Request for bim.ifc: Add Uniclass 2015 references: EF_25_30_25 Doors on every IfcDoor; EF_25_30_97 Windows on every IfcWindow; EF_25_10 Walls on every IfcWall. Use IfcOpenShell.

First a look at what the model holds.

```python
import ifcopenshell

model = ifcopenshell.open("bim.ifc")
print(model.schema)
print("classifications:", [c.Name for c in model.by_type("IfcClassification")])
for ifc_class in ("IfcDoor", "IfcRoof", "IfcStair", "IfcWall", "IfcWindow"):
    print(ifc_class, len(model.by_type(ifc_class)))
```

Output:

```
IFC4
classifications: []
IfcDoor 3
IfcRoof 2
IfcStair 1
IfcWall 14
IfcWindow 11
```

```python
import ifcopenshell
import ifcopenshell.api.classification

model = ifcopenshell.open("bim.ifc")

system = ifcopenshell.api.classification.add_classification(model, classification="Uniclass 2015")

codes = {
    "IfcDoor": ("EF_25_30_25", "Doors"),
    "IfcWindow": ("EF_25_30_97", "Windows"),
    "IfcWall": ("EF_25_10", "Walls"),
}
for ifc_class, (code, name) in codes.items():
    products = model.by_type(ifc_class)
    ifcopenshell.api.classification.add_reference(
        model, products=products, classification=system, identification=code, name=name
    )
    print(code, len(products))

model.write("bim_updated.ifc")
```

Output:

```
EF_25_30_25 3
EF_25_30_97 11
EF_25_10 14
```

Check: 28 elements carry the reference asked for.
